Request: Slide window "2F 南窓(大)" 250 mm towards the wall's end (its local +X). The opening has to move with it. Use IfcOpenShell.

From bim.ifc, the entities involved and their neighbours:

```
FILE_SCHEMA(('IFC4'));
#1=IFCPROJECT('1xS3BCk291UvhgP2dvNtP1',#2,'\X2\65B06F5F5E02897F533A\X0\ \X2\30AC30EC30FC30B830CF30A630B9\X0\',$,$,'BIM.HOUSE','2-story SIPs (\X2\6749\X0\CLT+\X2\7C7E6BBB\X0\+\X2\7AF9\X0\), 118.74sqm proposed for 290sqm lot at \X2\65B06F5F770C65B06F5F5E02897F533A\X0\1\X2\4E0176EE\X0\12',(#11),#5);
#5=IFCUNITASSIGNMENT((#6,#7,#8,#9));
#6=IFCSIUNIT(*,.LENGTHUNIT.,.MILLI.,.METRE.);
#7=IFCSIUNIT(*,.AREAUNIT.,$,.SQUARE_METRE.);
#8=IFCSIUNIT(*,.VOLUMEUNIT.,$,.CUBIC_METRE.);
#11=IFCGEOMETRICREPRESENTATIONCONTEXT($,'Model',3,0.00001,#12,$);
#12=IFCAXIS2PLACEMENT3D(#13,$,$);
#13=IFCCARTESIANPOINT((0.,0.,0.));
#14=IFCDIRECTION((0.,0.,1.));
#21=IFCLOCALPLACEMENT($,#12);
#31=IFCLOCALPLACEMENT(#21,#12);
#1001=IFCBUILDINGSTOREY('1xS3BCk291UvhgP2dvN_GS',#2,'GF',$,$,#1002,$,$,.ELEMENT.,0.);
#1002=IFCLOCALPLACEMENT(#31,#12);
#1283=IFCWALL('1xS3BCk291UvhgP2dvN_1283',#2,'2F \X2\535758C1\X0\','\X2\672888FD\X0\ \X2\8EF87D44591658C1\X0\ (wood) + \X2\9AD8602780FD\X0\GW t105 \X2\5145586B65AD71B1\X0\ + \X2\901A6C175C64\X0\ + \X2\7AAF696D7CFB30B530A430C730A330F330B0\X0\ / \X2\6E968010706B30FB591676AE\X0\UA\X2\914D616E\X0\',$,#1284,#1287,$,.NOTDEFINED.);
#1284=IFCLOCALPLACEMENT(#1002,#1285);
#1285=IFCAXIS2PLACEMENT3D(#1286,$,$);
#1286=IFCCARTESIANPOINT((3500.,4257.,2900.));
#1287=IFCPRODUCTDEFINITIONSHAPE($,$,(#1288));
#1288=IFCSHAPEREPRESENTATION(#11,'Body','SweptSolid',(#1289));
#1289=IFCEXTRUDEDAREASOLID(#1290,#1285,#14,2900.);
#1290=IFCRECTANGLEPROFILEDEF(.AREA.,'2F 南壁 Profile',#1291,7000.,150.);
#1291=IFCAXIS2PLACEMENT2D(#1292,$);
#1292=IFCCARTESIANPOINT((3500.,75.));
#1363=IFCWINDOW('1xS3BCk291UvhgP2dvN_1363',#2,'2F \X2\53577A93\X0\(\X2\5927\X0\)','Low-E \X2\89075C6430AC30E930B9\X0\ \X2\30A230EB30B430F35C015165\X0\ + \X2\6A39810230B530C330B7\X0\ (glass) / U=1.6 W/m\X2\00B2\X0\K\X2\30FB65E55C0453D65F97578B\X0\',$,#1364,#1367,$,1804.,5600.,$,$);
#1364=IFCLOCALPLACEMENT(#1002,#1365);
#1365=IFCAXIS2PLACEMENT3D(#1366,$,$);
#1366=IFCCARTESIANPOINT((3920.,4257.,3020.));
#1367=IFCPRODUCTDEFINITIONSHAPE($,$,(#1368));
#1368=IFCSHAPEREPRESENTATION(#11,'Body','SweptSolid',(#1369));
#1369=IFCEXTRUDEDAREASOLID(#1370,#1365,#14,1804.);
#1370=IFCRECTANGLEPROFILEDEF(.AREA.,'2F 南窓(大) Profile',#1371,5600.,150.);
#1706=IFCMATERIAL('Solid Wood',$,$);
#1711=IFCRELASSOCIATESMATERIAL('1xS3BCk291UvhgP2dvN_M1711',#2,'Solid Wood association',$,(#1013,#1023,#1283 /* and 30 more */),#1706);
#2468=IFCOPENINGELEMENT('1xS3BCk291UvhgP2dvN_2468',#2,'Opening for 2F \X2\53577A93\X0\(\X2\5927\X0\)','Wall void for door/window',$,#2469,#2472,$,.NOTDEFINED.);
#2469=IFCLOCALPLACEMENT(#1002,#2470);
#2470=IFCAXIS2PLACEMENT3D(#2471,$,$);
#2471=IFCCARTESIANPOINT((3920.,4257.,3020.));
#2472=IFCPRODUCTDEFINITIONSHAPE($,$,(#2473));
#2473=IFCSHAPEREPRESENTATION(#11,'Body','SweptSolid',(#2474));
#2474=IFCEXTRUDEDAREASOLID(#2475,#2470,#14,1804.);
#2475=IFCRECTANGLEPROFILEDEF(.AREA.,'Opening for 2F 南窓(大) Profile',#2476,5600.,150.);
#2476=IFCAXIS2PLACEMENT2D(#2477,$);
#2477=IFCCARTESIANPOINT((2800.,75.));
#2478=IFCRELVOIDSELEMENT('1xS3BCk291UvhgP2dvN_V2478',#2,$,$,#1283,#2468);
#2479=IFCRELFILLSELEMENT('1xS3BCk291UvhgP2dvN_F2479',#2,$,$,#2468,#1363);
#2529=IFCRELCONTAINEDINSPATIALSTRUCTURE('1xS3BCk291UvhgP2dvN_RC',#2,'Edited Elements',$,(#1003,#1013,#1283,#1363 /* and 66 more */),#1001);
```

```python
import ifcopenshell
import ifcopenshell.api.geometry
import ifcopenshell.util.placement

model = ifcopenshell.open("bim.ifc")

window = model.by_guid("1xS3BCk291UvhgP2dvN_1363")
opening = window.FillsVoids[0].RelatingOpeningElement
wall = opening.VoidsElements[0].RelatingBuildingElement

wall_matrix = ifcopenshell.util.placement.get_local_placement(wall.ObjectPlacement)
shift = wall_matrix[:3, 0] * 250.0
before = ifcopenshell.util.placement.get_local_placement(window.ObjectPlacement)[:3, 3].copy()

# The window is not placed relative to its opening, so move both.
for product in (opening, window):
    matrix = ifcopenshell.util.placement.get_local_placement(product.ObjectPlacement)
    matrix[:3, 3] += shift
    ifcopenshell.api.geometry.edit_object_placement(model, product=product, matrix=matrix, is_si=False)

after = ifcopenshell.util.placement.get_local_placement(window.ObjectPlacement)[:3, 3]
print("window moved by", (after - before).round(3) + 0.0)

model.write("bim_edited.ifc")
```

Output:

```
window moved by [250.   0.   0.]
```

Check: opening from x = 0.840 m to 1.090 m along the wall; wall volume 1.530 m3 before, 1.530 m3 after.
